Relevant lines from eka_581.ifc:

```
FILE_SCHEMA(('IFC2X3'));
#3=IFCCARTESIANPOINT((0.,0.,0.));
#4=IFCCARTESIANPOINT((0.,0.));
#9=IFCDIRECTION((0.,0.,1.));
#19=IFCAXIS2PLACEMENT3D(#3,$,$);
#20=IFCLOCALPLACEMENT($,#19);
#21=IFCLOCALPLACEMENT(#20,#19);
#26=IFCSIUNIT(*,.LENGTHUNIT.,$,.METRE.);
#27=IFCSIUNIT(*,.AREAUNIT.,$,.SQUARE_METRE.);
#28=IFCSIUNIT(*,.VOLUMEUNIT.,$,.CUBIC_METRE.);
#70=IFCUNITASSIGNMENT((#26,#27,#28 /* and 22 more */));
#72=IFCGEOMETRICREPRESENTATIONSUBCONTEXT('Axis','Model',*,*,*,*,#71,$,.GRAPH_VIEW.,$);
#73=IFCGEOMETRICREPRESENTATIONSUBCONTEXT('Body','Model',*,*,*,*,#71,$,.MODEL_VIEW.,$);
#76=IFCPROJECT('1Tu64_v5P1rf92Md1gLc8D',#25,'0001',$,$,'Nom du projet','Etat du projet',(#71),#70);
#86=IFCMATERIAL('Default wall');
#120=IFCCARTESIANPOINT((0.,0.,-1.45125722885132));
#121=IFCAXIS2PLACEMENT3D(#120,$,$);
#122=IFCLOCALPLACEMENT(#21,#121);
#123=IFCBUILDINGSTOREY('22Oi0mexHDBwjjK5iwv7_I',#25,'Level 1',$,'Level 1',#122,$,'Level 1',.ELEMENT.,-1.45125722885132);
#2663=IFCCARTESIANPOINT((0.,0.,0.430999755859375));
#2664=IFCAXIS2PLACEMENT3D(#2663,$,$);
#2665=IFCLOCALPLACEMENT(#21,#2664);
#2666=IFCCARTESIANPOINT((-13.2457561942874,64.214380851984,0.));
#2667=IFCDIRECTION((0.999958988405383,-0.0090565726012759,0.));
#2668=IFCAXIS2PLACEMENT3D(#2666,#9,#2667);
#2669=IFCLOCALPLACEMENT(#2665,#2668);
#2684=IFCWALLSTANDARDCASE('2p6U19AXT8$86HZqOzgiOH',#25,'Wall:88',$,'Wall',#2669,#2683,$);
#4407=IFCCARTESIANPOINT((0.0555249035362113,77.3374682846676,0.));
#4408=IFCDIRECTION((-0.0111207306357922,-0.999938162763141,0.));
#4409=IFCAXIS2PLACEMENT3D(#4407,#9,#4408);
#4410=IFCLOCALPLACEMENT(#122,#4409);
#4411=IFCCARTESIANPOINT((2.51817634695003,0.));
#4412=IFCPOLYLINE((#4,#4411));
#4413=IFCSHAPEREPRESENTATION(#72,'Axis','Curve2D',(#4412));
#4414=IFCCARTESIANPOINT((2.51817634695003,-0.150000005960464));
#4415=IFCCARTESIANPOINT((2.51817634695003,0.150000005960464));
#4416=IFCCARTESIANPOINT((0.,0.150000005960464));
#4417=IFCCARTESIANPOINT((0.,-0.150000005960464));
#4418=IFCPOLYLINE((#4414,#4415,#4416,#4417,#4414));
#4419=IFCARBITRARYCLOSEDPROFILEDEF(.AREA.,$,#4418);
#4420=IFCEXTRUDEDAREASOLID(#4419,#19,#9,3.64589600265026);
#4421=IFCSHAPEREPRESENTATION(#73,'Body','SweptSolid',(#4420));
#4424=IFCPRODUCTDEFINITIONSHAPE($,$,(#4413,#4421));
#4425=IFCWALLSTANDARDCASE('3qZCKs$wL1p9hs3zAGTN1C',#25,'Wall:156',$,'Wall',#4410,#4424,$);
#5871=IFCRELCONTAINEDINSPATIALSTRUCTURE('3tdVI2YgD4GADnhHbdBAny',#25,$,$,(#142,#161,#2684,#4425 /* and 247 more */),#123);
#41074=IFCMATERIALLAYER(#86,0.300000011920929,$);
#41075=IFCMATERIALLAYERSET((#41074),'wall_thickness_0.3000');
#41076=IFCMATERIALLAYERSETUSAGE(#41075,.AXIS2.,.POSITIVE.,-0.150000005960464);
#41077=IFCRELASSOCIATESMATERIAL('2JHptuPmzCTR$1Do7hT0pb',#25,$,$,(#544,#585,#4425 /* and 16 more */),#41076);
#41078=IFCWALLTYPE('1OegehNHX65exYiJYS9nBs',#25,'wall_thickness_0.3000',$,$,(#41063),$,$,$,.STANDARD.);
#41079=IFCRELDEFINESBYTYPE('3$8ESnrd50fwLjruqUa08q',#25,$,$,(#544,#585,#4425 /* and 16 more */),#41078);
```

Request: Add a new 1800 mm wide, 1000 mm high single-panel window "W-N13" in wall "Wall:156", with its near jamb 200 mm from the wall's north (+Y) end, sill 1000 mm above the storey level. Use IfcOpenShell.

```python
import numpy as np
import ifcopenshell
import ifcopenshell.api.feature
import ifcopenshell.api.geometry
import ifcopenshell.api.root
import ifcopenshell.api.spatial
import ifcopenshell.api.type
import ifcopenshell.geom
import ifcopenshell.util.element
import ifcopenshell.util.placement
import ifcopenshell.util.representation
import ifcopenshell.util.shape
import ifcopenshell.util.unit

model = ifcopenshell.open("eka_581.ifc")
unit_scale = ifcopenshell.util.unit.calculate_unit_scale(model)
settings = ifcopenshell.geom.settings()


def volume(element):
    """Net volume in cubic metres, openings subtracted."""
    shape = ifcopenshell.geom.create_shape(settings, element)
    return ifcopenshell.util.shape.get_volume(shape.geometry)


wall = model.by_guid("3qZCKs$wL1p9hs3zAGTN1C")
storey = ifcopenshell.util.element.get_container(wall, ifc_class="IfcBuildingStorey")
context = ifcopenshell.util.representation.get_context(model, "Model", "Body", "MODEL_VIEW")
before = volume(wall)

width, height, from_end, sill = 1.8, 1, 0.2, 1  # metres

# The wall runs along its own X axis, and the end named is its -X end.
wall_shape = ifcopenshell.geom.create_shape(settings, wall)
x, y, z = ifcopenshell.util.shape.get_vertices(wall_shape.geometry).T
start = x.min() + from_end
face, thickness = float(y.min()), float(y.max() - y.min())
wall_matrix = ifcopenshell.util.placement.get_local_placement(wall.ObjectPlacement)
level = ifcopenshell.util.placement.get_local_placement(storey.ObjectPlacement)[2, 3]


def in_wall(x, y):
    """Placement at x, y metres in the wall's axes, at sill height."""
    matrix = wall_matrix.copy()
    matrix[:, 3] = wall_matrix @ np.array([x / unit_scale, y / unit_scale, 0.0, 1.0])
    matrix[2, 3] = level + sill / unit_scale
    return matrix


# Opening: a box that overshoots both wall faces by 50 mm.
opening = ifcopenshell.api.root.create_entity(model, ifc_class="IfcOpeningElement")
box = ifcopenshell.api.geometry.add_wall_representation(
    model, context=context, length=width, height=height, thickness=thickness + 0.1
)
ifcopenshell.api.geometry.assign_representation(model, product=opening, representation=box)
ifcopenshell.api.geometry.edit_object_placement(model, product=opening, matrix=in_wall(start, face - 0.05), is_si=False)
ifcopenshell.api.feature.add_feature(model, feature=opening, element=wall)

window = ifcopenshell.api.root.create_entity(model, ifc_class="IfcWindow", name="W-N13")
window.OverallWidth, window.OverallHeight = width / unit_scale, height / unit_scale
body = ifcopenshell.api.geometry.add_window_representation(
    model,
    context=context,
    overall_width=window.OverallWidth,
    overall_height=window.OverallHeight,
    partition_type="SINGLE_PANEL",
)
ifcopenshell.api.geometry.assign_representation(model, product=window, representation=body)
ifcopenshell.api.spatial.assign_container(model, products=[window], relating_structure=storey)
fills = ifcopenshell.api.feature.add_filling(model, opening=opening, element=window)
fills.OwnerHistory = window.OwnerHistory  # required in IFC2X3

# IFC2X3 keeps the operation on the window style.
style = ifcopenshell.api.root.create_entity(model, ifc_class="IfcWindowStyle", name="W-N13")
style.OperationType, style.ConstructionType = "SINGLE_PANEL", "NOTDEFINED"
style.ParameterTakesPrecedence = style.Sizeable = False
ifcopenshell.api.type.assign_type(model, related_objects=[window], relating_type=style)

# Centre the window in the wall's thickness.
ifcopenshell.api.geometry.edit_object_placement(model, product=window, matrix=in_wall(start, face), is_si=False)
window_shape = ifcopenshell.geom.create_shape(settings, window)
depth = ifcopenshell.util.shape.get_vertices(window_shape.geometry)[:, 1]
offset = face + thickness / 2 - (depth.min() + depth.max()) / 2
ifcopenshell.api.geometry.edit_object_placement(model, product=window, matrix=in_wall(start, offset), is_si=False)

after = volume(wall)

print(f"wall volume {before:.3f} -> {after:.3f} m3")

model.write("eka_581_updated.ifc")
```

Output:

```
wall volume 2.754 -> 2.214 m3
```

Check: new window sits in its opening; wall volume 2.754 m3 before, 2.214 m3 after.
